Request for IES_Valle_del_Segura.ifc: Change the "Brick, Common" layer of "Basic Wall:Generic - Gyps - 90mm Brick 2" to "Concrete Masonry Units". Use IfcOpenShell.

First a look at what the model holds.

```python
import ifcopenshell
import ifcopenshell.util.element

model = ifcopenshell.open("IES_Valle_del_Segura.ifc")
print(model.schema)
for layer_set in model.by_type("IfcMaterialLayerSet"):
    if layer_set.LayerSetName == "Basic Wall:Generic - Gyps - 90mm Brick 2":
        for layer in layer_set.MaterialLayers:
            print(layer.id(), layer.Material and layer.Material.Name, layer.LayerThickness, sep=" | ")
        print(len(ifcopenshell.util.element.get_elements_by_material(model, layer_set)), "elements and types use it")
print(sorted(m.Name for m in model.by_type("IfcMaterial") if m.Name)[:60])
```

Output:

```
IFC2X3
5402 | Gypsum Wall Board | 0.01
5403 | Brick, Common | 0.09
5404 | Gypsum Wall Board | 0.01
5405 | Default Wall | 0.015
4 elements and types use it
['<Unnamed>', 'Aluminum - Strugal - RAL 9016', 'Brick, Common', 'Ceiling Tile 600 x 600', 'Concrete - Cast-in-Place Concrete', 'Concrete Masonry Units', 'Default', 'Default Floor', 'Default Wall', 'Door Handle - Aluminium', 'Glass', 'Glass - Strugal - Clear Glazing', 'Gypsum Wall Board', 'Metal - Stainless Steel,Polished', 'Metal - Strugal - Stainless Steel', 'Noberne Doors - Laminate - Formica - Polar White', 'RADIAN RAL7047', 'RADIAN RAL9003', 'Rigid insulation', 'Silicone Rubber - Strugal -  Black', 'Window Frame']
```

```python
import ifcopenshell
import ifcopenshell.api.material

model = ifcopenshell.open("IES_Valle_del_Segura.ifc")

layer_set = next(s for s in model.by_type("IfcMaterialLayerSet") if s.LayerSetName == "Basic Wall:Generic - Gyps - 90mm Brick 2")
layer = next(l for l in layer_set.MaterialLayers if l.Material and l.Material.Name == "Brick, Common")
material = next(m for m in model.by_type("IfcMaterial") if m.Name == "Concrete Masonry Units")

# Point this one layer at the other material; renaming the old one would change it everywhere.
ifcopenshell.api.material.edit_layer(model, layer=layer, attributes={}, material=material)

print([l.Material.Name if l.Material else None for l in layer_set.MaterialLayers])

model.write("IES_Valle_del_Segura_rev.ifc")
```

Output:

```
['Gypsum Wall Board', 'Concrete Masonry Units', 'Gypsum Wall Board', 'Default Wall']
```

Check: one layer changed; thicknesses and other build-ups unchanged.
